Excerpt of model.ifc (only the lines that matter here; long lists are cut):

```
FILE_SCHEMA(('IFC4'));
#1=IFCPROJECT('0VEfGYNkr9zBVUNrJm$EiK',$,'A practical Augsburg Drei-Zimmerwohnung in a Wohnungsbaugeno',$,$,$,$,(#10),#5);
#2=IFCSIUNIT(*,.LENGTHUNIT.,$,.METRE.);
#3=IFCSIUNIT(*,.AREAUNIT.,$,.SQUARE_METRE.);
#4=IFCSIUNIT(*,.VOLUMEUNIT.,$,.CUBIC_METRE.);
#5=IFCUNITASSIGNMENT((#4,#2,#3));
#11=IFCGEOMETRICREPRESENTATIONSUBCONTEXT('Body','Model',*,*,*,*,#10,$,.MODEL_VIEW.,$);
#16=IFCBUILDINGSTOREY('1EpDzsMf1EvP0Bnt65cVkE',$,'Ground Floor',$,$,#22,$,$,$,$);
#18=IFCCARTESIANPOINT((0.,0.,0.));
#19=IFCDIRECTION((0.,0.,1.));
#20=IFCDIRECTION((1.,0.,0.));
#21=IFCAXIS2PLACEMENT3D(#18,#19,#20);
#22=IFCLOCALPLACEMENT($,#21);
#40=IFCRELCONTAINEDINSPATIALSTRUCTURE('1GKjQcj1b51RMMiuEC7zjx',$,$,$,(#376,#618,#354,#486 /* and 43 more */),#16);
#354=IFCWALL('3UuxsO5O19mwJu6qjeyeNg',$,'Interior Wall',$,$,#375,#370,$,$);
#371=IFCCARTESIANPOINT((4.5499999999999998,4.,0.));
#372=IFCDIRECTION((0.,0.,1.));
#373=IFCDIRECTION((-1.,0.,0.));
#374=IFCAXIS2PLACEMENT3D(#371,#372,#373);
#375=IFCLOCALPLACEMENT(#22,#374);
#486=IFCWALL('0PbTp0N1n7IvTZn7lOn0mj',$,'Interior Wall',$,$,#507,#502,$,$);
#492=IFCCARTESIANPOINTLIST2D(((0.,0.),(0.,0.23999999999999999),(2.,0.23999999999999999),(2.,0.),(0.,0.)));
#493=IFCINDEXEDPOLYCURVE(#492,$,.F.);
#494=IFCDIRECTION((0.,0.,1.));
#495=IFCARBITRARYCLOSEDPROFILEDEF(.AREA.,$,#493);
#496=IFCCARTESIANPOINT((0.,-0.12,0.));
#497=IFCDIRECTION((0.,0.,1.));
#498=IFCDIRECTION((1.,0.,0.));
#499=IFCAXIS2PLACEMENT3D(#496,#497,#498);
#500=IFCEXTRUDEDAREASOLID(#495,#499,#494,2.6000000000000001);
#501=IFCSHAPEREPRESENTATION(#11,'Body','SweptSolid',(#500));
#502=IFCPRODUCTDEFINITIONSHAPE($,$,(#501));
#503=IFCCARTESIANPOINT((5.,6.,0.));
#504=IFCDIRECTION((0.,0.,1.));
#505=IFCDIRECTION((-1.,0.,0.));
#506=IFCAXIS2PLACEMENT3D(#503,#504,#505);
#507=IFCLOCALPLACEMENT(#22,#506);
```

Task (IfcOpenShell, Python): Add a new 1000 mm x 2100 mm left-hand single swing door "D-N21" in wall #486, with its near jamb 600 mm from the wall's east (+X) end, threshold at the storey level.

```python
import numpy as np
import ifcopenshell
import ifcopenshell.api.feature
import ifcopenshell.api.geometry
import ifcopenshell.api.root
import ifcopenshell.api.spatial
import ifcopenshell.geom
import ifcopenshell.util.element
import ifcopenshell.util.placement
import ifcopenshell.util.representation
import ifcopenshell.util.shape
import ifcopenshell.util.unit

model = ifcopenshell.open("model.ifc")
unit_scale = ifcopenshell.util.unit.calculate_unit_scale(model)
settings = ifcopenshell.geom.settings()


def volume(element):
    """Net volume in cubic metres, openings subtracted."""
    shape = ifcopenshell.geom.create_shape(settings, element)
    return ifcopenshell.util.shape.get_volume(shape.geometry)


wall = model.by_id(486)
storey = ifcopenshell.util.element.get_container(wall, ifc_class="IfcBuildingStorey")
context = ifcopenshell.util.representation.get_context(model, "Model", "Body", "MODEL_VIEW")
before = volume(wall)

width, height, from_end, sill = 1, 2.1, 0.6, 0.0  # metres

# The wall runs along its own X axis, and the end named is its -X end.
wall_shape = ifcopenshell.geom.create_shape(settings, wall)
x, y, z = ifcopenshell.util.shape.get_vertices(wall_shape.geometry).T
start = x.min() + from_end
face, thickness = float(y.min()), float(y.max() - y.min())
wall_matrix = ifcopenshell.util.placement.get_local_placement(wall.ObjectPlacement)
level = ifcopenshell.util.placement.get_local_placement(storey.ObjectPlacement)[2, 3]


def in_wall(x, y):
    """Placement at x, y metres in the wall's axes, at sill height."""
    matrix = wall_matrix.copy()
    matrix[:, 3] = wall_matrix @ np.array([x / unit_scale, y / unit_scale, 0.0, 1.0])
    matrix[2, 3] = level + sill / unit_scale
    return matrix


# Opening: a box that overshoots both wall faces by 50 mm.
opening = ifcopenshell.api.root.create_entity(model, ifc_class="IfcOpeningElement", predefined_type="OPENING")
box = ifcopenshell.api.geometry.add_wall_representation(
    model, context=context, length=width, height=height, thickness=thickness + 0.1
)
ifcopenshell.api.geometry.assign_representation(model, product=opening, representation=box)
ifcopenshell.api.geometry.edit_object_placement(model, product=opening, matrix=in_wall(start, face - 0.05), is_si=False)
ifcopenshell.api.feature.add_feature(model, feature=opening, element=wall)

door = ifcopenshell.api.root.create_entity(model, ifc_class="IfcDoor", name="D-N21", predefined_type="DOOR")
door.OverallWidth, door.OverallHeight = width / unit_scale, height / unit_scale
door.OperationType = "SINGLE_SWING_LEFT"
body = ifcopenshell.api.geometry.add_door_representation(
    model,
    context=context,
    overall_width=door.OverallWidth,
    overall_height=door.OverallHeight,
    operation_type="SINGLE_SWING_LEFT",
    lining_properties={"LiningDepth": thickness / unit_scale, "ThresholdDepth": thickness / unit_scale},
)
ifcopenshell.api.geometry.assign_representation(model, product=door, representation=body)
ifcopenshell.api.spatial.assign_container(model, products=[door], relating_structure=storey)
ifcopenshell.api.feature.add_filling(model, opening=opening, element=door)

# The lining spans the wall, so the door starts at the wall face.
ifcopenshell.api.geometry.edit_object_placement(model, product=door, matrix=in_wall(start, face), is_si=False)

after = volume(wall)

print(f"wall volume {before:.3f} -> {after:.3f} m3")

model.write("model_updated.ifc")
```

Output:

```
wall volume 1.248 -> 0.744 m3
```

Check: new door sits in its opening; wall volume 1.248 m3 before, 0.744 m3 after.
